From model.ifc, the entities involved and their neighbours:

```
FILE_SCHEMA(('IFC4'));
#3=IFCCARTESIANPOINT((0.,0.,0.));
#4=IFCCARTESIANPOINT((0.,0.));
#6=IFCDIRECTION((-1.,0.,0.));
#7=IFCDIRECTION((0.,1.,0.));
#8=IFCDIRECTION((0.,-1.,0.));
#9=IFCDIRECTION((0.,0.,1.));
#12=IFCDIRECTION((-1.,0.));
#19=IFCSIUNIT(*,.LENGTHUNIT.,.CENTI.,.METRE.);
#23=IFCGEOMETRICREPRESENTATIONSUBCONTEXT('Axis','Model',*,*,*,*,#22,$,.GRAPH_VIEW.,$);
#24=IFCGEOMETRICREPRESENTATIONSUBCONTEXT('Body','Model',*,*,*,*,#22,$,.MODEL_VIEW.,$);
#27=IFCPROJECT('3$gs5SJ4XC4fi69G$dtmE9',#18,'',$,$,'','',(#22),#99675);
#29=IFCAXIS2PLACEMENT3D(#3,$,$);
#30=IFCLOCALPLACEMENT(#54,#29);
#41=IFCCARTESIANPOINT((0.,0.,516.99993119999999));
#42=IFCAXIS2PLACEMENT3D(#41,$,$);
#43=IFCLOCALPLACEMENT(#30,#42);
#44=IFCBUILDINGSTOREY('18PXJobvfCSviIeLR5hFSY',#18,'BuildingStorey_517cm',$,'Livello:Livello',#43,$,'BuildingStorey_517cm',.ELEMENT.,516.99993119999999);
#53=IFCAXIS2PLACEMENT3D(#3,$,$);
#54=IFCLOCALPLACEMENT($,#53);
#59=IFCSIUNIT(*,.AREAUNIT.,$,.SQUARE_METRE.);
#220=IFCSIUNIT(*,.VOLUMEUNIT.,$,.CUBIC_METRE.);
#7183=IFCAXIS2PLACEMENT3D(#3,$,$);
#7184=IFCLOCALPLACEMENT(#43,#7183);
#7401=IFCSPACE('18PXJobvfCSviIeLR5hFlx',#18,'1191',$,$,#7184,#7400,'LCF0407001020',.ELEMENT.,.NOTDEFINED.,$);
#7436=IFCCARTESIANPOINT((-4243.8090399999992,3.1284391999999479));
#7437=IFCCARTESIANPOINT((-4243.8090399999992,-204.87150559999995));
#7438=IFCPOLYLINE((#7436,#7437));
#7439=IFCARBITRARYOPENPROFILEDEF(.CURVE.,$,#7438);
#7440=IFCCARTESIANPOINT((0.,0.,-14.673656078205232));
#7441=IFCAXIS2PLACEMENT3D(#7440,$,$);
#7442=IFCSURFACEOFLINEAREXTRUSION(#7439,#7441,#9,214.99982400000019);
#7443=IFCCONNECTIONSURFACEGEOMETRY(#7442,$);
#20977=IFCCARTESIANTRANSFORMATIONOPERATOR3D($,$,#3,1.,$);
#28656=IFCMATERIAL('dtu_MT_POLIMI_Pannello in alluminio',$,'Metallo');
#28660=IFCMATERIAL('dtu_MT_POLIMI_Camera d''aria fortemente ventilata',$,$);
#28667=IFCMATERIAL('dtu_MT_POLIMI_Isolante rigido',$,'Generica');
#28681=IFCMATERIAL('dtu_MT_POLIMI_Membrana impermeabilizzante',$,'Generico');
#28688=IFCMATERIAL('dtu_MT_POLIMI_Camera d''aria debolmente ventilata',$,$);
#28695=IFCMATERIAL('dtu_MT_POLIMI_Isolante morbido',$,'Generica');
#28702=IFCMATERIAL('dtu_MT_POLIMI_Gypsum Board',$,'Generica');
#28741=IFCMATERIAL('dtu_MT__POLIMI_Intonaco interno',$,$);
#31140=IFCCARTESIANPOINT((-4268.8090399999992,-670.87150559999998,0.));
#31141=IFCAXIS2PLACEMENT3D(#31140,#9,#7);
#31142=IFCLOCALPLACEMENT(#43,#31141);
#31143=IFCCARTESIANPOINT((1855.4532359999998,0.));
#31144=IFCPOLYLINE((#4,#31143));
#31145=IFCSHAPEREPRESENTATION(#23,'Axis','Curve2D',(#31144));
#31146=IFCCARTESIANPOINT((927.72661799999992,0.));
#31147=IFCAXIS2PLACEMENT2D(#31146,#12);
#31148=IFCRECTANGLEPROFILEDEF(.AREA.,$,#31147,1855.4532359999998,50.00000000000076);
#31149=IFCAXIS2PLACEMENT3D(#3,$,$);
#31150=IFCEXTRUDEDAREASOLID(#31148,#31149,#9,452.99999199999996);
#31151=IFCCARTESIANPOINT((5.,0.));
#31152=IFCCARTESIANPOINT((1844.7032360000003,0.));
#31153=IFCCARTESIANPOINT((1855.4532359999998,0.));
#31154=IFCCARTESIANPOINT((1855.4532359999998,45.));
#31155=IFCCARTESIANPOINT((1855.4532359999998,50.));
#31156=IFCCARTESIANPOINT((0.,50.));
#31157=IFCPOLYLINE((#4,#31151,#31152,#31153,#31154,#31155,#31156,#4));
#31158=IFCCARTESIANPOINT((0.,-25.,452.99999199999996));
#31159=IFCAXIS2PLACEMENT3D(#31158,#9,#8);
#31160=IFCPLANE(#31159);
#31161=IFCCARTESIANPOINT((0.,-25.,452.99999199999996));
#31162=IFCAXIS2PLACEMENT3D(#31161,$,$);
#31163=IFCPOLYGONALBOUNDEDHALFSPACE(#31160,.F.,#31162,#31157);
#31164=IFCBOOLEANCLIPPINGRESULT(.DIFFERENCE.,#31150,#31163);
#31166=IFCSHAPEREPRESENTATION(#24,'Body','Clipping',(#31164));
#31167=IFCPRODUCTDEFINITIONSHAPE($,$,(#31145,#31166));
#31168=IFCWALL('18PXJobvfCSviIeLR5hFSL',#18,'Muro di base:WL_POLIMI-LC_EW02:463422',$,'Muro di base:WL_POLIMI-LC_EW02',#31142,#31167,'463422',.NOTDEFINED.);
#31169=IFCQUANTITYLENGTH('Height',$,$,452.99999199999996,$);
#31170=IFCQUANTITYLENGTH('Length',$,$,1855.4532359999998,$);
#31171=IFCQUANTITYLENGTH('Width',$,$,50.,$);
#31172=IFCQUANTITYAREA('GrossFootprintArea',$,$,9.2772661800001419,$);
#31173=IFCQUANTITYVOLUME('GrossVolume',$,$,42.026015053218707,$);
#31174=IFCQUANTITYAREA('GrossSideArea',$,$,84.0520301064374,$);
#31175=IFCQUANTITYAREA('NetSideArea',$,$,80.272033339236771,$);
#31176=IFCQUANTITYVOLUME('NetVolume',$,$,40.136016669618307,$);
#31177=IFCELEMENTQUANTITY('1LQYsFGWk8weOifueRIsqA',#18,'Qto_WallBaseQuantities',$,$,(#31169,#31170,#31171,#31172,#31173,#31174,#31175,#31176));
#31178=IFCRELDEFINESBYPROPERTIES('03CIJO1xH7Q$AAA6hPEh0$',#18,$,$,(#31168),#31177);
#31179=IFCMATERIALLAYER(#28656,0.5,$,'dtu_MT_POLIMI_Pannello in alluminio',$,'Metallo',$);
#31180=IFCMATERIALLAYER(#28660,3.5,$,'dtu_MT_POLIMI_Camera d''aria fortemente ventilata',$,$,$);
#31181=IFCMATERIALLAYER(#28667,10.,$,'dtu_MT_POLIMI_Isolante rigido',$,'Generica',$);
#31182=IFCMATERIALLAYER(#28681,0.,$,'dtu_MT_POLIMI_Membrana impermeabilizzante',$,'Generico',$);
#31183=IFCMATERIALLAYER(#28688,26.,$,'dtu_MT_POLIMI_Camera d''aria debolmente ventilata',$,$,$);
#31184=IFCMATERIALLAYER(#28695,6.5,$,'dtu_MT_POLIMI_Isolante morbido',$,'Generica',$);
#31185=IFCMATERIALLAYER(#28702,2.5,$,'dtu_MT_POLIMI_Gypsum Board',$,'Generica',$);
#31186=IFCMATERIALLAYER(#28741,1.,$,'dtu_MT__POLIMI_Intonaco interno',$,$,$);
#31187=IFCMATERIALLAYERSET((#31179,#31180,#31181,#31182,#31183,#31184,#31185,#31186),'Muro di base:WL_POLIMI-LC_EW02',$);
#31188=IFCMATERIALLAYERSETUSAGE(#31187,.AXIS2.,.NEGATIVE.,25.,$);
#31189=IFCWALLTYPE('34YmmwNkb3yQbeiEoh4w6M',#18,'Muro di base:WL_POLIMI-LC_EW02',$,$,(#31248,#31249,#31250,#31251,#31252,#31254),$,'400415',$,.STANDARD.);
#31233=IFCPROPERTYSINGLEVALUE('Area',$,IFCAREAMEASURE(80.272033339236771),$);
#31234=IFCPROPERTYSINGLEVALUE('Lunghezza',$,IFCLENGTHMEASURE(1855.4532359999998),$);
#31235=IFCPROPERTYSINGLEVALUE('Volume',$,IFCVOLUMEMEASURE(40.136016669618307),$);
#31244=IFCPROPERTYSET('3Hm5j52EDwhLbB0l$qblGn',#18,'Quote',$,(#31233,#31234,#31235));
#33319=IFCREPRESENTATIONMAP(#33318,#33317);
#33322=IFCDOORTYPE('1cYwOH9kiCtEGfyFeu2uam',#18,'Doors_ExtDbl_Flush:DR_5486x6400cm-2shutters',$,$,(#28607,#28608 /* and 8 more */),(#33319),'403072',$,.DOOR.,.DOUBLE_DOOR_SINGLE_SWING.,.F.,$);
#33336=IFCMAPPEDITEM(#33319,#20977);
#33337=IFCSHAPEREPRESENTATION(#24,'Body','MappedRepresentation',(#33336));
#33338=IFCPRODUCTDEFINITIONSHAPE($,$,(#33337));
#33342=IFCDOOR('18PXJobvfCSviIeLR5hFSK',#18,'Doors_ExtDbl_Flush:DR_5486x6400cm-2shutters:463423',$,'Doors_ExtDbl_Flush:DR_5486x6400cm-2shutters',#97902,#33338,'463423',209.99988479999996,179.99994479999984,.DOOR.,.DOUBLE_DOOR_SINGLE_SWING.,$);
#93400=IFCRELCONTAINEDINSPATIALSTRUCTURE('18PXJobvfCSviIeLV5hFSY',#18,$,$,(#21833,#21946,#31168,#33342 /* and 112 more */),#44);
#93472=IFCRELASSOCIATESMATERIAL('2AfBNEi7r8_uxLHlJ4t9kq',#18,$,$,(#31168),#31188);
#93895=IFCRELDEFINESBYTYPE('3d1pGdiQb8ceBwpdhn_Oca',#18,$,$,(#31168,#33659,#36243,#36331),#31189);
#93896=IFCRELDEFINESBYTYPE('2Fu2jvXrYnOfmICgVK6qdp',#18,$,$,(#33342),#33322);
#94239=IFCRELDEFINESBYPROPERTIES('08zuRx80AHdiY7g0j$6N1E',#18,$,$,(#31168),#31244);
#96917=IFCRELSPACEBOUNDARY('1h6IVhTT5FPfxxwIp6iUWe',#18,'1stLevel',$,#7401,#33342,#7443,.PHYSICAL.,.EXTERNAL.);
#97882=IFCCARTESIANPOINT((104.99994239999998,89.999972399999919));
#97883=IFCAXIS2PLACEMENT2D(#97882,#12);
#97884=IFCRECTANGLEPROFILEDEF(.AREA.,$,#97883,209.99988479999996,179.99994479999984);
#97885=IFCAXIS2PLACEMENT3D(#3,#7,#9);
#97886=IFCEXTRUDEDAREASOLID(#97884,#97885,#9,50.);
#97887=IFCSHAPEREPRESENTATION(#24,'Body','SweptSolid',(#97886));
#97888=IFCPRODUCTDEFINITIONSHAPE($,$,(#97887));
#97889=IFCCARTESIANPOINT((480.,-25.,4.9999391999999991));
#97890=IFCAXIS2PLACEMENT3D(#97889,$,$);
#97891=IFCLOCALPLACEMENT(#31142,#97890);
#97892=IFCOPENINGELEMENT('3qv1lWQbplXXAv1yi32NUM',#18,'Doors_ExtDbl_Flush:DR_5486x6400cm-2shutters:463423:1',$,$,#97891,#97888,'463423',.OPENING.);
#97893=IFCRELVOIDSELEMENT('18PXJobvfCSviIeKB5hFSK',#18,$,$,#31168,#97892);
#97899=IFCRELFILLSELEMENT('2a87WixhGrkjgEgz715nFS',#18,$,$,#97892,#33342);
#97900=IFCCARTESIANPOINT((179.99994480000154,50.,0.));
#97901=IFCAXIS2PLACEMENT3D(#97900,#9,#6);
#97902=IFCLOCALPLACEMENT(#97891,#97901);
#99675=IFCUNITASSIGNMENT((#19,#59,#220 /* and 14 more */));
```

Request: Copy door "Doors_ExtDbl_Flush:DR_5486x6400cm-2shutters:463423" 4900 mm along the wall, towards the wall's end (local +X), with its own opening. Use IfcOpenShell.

```python
import numpy as np
import ifcopenshell
import ifcopenshell.api.feature
import ifcopenshell.api.geometry
import ifcopenshell.api.pset
import ifcopenshell.api.root
import ifcopenshell.geom
import ifcopenshell.util.element
import ifcopenshell.util.placement
import ifcopenshell.util.shape
import ifcopenshell.util.unit

model = ifcopenshell.open("model.ifc")
unit_scale = ifcopenshell.util.unit.calculate_unit_scale(model)
area_scale = ifcopenshell.util.unit.calculate_unit_scale(model, "AREAUNIT")
volume_scale = ifcopenshell.util.unit.calculate_unit_scale(model, "VOLUMEUNIT")
settings = ifcopenshell.geom.settings()


def volume(element):
    """Net volume in cubic metres, openings subtracted."""
    shape = ifcopenshell.geom.create_shape(settings, element)
    return ifcopenshell.util.shape.get_volume(shape.geometry)


def reuse_history(source, copy):
    """copy_class also copies each property set's owner history, people and application; keep the originals."""
    for rel in copy.IsDefinedBy:
        if rel.is_a("IfcRelDefinesByProperties") and (history := rel.RelatingPropertyDefinition.OwnerHistory):
            rel.RelatingPropertyDefinition.OwnerHistory = source.OwnerHistory
            ifcopenshell.util.element.remove_deep2(model, history)


door = model.by_guid("18PXJobvfCSviIeLR5hFSK")
opening = door.FillsVoids[0].RelatingOpeningElement
wall = opening.VoidsElements[0].RelatingBuildingElement
before = volume(wall)
shift = ifcopenshell.util.placement.get_local_placement(wall.ObjectPlacement)[:3, 0] * 4.9 / unit_scale

# copy_class copies the void relationship, type, container and properties, but no geometry.
new_opening = ifcopenshell.api.root.copy_class(model, product=opening)
new_opening.Representation = ifcopenshell.util.element.copy_deep(
    model, opening.Representation, exclude=["IfcGeometricRepresentationContext", "IfcRepresentationMap"]
)
new_opening.Name = "Doors_ExtDbl_Flush:DR_5486x6400cm-2shutters"
new_opening.Tag = None
reuse_history(opening, new_opening)
new_door = ifcopenshell.api.root.copy_class(model, product=door)
new_door.Representation = ifcopenshell.util.element.copy_deep(
    model, door.Representation, exclude=["IfcGeometricRepresentationContext", "IfcRepresentationMap"]
)
new_door.Name = "Doors_ExtDbl_Flush:DR_5486x6400cm-2shutters"
new_door.Tag = None
reuse_history(door, new_door)
ifcopenshell.api.feature.add_filling(model, opening=new_opening, element=new_door)

for old, new in ((opening, new_opening), (door, new_door)):
    matrix = ifcopenshell.util.placement.get_local_placement(old.ObjectPlacement)
    matrix[:3, 3] += shift
    ifcopenshell.api.geometry.edit_object_placement(model, product=new, matrix=matrix, is_si=False)

# The copied space boundaries still share their surfaces with the original.
for rel in new_door.ProvidesBoundaries:
    if rel.ConnectionGeometry:
        rel.ConnectionGeometry = ifcopenshell.util.element.copy_deep(model, rel.ConnectionGeometry)

# Space boundary surfaces are stored in each space's coordinates; move them too.
for rel in new_door.ProvidesBoundaries:
    if not rel.ConnectionGeometry:
        continue
    surface = rel.ConnectionGeometry.SurfaceOnRelatingElement
    space_matrix = ifcopenshell.util.placement.get_local_placement(rel.RelatingSpace.ObjectPlacement)
    point = np.array(surface.Position.Location.Coordinates) + space_matrix[:3, :3].T @ shift
    surface.Position = model.createIfcAxis2Placement3D(
        model.createIfcCartesianPoint(point.tolist()), surface.Position.Axis, surface.Position.RefDirection
    )

after = volume(wall)
thickness = 0.5  # wall thickness in metres

# Update the wall's stored quantities.
qto = model.by_id(ifcopenshell.util.element.get_pset(wall, "Qto_WallBaseQuantities", should_inherit=False)["id"])
ifcopenshell.api.pset.edit_qto(model, qto=qto, properties={
    "NetSideArea": after / thickness / area_scale,
    "NetVolume": after / volume_scale,
})
pset = model.by_id(ifcopenshell.util.element.get_pset(wall, "Quote", should_inherit=False)["id"])
ifcopenshell.api.pset.edit_pset(model, pset=pset, properties={
    "Area": model.create_entity("IfcAreaMeasure", after / thickness / area_scale),
    "Volume": model.create_entity("IfcVolumeMeasure", after / volume_scale),
})

print(f"wall volume {before:.3f} -> {after:.3f} m3")

model.write("model_v2.ifc")
```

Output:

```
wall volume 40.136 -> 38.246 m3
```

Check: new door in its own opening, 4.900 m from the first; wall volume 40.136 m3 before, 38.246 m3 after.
